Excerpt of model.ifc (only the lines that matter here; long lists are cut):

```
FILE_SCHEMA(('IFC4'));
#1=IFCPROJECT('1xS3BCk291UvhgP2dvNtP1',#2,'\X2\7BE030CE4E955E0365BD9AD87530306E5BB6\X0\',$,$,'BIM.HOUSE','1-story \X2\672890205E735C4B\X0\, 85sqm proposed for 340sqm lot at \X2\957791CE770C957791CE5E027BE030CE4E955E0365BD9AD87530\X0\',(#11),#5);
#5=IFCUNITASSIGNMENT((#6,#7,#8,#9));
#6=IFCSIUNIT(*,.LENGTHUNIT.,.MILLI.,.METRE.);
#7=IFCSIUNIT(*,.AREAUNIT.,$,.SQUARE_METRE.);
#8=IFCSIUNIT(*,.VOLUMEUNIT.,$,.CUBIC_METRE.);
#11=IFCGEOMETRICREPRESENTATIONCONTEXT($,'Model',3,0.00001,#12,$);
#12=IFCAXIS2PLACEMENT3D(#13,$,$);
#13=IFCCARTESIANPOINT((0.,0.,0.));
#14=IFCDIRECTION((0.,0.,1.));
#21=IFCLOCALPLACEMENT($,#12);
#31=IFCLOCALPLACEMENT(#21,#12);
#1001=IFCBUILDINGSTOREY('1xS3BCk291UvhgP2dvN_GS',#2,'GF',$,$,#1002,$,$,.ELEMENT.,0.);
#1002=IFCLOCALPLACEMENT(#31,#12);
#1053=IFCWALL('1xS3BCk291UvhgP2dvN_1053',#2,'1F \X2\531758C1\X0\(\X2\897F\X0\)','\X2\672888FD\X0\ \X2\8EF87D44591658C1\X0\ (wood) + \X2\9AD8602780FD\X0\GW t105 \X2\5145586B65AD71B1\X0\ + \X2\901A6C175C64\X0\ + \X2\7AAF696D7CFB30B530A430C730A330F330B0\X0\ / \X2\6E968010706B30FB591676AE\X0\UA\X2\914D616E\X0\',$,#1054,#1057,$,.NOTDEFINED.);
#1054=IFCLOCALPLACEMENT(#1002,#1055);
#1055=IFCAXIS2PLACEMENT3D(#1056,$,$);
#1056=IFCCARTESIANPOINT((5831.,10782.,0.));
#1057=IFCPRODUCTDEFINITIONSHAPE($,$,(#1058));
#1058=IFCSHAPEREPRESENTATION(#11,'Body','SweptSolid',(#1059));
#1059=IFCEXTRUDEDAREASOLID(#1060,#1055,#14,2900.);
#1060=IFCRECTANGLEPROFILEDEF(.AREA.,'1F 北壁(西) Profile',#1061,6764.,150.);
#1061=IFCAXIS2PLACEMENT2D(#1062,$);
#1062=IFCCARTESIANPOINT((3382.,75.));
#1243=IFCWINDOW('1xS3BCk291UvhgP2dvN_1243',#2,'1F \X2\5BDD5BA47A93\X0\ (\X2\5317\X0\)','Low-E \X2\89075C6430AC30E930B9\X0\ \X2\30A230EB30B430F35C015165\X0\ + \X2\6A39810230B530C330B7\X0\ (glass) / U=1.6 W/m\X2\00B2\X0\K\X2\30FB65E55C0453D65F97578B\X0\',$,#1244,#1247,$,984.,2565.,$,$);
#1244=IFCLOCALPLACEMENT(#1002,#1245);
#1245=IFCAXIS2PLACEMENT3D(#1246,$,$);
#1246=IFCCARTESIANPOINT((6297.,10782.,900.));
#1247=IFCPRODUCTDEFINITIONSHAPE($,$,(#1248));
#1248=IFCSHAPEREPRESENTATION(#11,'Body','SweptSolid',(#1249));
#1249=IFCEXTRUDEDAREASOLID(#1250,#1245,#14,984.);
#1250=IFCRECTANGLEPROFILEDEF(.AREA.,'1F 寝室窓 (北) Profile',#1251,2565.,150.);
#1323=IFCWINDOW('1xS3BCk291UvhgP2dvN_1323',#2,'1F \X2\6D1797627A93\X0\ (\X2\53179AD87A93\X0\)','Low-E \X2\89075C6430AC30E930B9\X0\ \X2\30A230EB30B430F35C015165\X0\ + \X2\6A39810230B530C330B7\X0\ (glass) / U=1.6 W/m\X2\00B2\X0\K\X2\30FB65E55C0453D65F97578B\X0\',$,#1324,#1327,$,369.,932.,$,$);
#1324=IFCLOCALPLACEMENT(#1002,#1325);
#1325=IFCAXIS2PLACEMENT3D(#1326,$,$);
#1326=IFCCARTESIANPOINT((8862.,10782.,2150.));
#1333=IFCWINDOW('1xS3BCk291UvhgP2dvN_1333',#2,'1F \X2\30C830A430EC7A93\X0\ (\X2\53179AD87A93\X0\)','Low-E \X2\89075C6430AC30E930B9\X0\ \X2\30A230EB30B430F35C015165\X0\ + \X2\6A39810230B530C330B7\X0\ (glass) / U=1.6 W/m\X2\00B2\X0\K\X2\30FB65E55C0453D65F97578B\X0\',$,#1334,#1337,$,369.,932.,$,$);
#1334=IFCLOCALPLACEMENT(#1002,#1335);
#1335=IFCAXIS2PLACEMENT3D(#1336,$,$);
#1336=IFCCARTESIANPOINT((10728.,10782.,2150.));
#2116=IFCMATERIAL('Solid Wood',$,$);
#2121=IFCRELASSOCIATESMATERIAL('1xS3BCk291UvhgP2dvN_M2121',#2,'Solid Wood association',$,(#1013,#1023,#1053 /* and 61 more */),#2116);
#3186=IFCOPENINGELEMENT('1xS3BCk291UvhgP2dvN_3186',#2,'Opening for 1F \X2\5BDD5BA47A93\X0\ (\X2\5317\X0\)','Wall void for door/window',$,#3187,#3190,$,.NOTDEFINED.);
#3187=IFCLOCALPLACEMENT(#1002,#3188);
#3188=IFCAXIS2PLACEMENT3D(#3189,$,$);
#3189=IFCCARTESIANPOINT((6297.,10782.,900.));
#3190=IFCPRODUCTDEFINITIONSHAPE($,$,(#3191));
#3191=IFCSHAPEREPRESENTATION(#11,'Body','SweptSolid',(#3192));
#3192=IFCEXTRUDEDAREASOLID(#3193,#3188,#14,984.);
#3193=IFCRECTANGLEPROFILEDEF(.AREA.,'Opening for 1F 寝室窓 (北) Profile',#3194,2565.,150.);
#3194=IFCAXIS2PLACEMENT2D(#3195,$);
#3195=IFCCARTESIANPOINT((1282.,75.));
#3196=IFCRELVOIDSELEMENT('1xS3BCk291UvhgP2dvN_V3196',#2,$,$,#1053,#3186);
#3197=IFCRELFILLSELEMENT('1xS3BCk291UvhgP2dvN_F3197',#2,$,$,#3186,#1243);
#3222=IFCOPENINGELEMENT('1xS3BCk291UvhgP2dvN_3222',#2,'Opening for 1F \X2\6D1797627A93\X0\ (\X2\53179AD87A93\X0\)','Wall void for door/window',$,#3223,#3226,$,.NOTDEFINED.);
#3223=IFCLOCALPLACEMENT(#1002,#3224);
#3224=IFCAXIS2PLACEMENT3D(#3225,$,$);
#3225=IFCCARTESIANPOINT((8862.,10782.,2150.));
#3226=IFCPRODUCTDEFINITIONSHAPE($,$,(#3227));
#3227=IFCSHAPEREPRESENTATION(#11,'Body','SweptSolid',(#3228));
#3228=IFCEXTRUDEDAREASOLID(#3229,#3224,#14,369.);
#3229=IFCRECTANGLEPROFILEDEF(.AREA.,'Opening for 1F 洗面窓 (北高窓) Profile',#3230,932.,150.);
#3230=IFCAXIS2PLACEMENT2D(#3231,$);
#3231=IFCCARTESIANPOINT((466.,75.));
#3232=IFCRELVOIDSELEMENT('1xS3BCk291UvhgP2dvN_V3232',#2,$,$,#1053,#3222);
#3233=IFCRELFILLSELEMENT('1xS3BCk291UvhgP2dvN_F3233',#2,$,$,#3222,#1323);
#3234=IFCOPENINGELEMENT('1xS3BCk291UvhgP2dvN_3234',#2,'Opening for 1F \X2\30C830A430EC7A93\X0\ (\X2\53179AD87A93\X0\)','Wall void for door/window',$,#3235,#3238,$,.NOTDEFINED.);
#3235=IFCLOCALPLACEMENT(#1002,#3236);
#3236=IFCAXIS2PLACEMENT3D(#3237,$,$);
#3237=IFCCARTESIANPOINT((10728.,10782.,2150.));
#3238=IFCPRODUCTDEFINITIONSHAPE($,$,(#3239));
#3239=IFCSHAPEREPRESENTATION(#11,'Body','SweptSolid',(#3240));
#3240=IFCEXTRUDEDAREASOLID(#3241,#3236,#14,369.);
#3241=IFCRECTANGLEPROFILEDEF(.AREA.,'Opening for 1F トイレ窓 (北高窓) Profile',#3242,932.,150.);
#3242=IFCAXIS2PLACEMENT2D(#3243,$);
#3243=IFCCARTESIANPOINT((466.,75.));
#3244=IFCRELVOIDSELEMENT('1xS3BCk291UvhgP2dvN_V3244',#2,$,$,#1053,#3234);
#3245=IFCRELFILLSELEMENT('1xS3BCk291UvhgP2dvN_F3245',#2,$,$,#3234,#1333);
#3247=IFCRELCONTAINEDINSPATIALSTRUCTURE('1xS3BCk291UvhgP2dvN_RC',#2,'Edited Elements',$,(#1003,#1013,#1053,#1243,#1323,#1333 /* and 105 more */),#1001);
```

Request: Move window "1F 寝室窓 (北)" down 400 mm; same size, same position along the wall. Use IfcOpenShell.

```python
import numpy as np
import ifcopenshell
import ifcopenshell.api.geometry
import ifcopenshell.util.placement
import ifcopenshell.util.unit

model = ifcopenshell.open("model.ifc")
unit_scale = ifcopenshell.util.unit.calculate_unit_scale(model)

window = model.by_id(1243)
opening = window.FillsVoids[0].RelatingOpeningElement
dz = -400.0

shift = np.array([0.0, 0.0, dz])
# The window is not placed relative to its opening, so move both.
for product in (opening, window):
    matrix = ifcopenshell.util.placement.get_local_placement(product.ObjectPlacement)
    matrix[:3, 3] += shift
    ifcopenshell.api.geometry.edit_object_placement(model, product=product, matrix=matrix, is_si=False)

print(f"moved by {dz * unit_scale:+.3f} m")

model.write("model_edited.ifc")
```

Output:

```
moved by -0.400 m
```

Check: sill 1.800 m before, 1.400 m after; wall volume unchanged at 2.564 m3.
